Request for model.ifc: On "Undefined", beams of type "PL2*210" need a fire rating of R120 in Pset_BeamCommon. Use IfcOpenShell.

First a look at what the model holds.

```python
import ifcopenshell
import ifcopenshell.util.element

model = ifcopenshell.open("model.ifc")
print(model.schema)
storey = next(s for s in model.by_type("IfcBuildingStorey") if s.Name == "Undefined")
beams = [e for e in ifcopenshell.util.element.get_decomposition(storey) if e.is_a("IfcBeam")]
seen = {}
for e in beams:
    element_type = ifcopenshell.util.element.get_type(e)
    key = (element_type.Name if element_type != e and element_type else None, ifcopenshell.util.element.get_pset(e, "Pset_BeamCommon", "FireRating"))
    seen[key] = seen.get(key, 0) + 1
for (name, value), count in sorted(seen.items(), key=str):
    print(count, "x", name, "|", value)
```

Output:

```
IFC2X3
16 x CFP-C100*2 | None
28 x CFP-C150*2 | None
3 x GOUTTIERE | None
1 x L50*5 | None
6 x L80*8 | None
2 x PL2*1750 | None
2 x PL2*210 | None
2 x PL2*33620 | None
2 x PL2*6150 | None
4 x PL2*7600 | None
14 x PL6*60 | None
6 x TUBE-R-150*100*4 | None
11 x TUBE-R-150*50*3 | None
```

```python
import ifcopenshell
import ifcopenshell.api.pset
import ifcopenshell.util.element

model = ifcopenshell.open("model.ifc")

storey = next(s for s in model.by_type("IfcBuildingStorey") if s.Name == "Undefined")
beams = [e for e in ifcopenshell.util.element.get_decomposition(storey) if e.is_a("IfcBeam")]

count = 0
for e in beams:
    element_type = ifcopenshell.util.element.get_type(e)
    if element_type in (None, e) or element_type.Name != "PL2*210":
        continue
    # add_pset returns the element's existing set when there is one.
    pset = ifcopenshell.api.pset.add_pset(model, product=e, name="Pset_BeamCommon")
    ifcopenshell.api.pset.edit_pset(model, pset=pset, properties={"FireRating": "R120"})
    count += 1

print(count, "beams updated")

model.write("model_updated.ifc")
```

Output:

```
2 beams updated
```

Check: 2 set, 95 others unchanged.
